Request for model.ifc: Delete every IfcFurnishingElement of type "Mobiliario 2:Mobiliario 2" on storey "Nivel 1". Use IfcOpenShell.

First a look at what the model holds.

```python
import ifcopenshell
import ifcopenshell.util.element

model = ifcopenshell.open("model.ifc")
print(model.schema)
storey = next(s for s in model.by_type("IfcBuildingStorey") if s.Name == "Nivel 1")
furniture = [e for e in ifcopenshell.util.element.get_decomposition(storey) if e.is_a("IfcFurnishingElement")]
seen = {}
for e in furniture:
    element_type = ifcopenshell.util.element.get_type(e)
    name = element_type.Name if element_type not in (None, e) else None
    seen[name] = seen.get(name, 0) + 1
for name, count in sorted(seen.items(), key=str):
    print(count, "x", name)
```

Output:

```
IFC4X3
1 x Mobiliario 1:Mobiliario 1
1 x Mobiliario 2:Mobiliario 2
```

```python
import ifcopenshell
import ifcopenshell.api.root
import ifcopenshell.util.element

model = ifcopenshell.open("model.ifc")

storey = next(s for s in model.by_type("IfcBuildingStorey") if s.Name == "Nivel 1")
furniture = [e for e in ifcopenshell.util.element.get_decomposition(storey) if e.is_a("IfcFurnishingElement")]
targets = [e for e in furniture if (t := ifcopenshell.util.element.get_type(e)) not in (None, e) and t.Name == "Mobiliario 2:Mobiliario 2"]

for e in targets:
    ifcopenshell.api.root.remove_product(model, product=e)
print(len(targets), "removed")

model.write("model_updated.ifc")
```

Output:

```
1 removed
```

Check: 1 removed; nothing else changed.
